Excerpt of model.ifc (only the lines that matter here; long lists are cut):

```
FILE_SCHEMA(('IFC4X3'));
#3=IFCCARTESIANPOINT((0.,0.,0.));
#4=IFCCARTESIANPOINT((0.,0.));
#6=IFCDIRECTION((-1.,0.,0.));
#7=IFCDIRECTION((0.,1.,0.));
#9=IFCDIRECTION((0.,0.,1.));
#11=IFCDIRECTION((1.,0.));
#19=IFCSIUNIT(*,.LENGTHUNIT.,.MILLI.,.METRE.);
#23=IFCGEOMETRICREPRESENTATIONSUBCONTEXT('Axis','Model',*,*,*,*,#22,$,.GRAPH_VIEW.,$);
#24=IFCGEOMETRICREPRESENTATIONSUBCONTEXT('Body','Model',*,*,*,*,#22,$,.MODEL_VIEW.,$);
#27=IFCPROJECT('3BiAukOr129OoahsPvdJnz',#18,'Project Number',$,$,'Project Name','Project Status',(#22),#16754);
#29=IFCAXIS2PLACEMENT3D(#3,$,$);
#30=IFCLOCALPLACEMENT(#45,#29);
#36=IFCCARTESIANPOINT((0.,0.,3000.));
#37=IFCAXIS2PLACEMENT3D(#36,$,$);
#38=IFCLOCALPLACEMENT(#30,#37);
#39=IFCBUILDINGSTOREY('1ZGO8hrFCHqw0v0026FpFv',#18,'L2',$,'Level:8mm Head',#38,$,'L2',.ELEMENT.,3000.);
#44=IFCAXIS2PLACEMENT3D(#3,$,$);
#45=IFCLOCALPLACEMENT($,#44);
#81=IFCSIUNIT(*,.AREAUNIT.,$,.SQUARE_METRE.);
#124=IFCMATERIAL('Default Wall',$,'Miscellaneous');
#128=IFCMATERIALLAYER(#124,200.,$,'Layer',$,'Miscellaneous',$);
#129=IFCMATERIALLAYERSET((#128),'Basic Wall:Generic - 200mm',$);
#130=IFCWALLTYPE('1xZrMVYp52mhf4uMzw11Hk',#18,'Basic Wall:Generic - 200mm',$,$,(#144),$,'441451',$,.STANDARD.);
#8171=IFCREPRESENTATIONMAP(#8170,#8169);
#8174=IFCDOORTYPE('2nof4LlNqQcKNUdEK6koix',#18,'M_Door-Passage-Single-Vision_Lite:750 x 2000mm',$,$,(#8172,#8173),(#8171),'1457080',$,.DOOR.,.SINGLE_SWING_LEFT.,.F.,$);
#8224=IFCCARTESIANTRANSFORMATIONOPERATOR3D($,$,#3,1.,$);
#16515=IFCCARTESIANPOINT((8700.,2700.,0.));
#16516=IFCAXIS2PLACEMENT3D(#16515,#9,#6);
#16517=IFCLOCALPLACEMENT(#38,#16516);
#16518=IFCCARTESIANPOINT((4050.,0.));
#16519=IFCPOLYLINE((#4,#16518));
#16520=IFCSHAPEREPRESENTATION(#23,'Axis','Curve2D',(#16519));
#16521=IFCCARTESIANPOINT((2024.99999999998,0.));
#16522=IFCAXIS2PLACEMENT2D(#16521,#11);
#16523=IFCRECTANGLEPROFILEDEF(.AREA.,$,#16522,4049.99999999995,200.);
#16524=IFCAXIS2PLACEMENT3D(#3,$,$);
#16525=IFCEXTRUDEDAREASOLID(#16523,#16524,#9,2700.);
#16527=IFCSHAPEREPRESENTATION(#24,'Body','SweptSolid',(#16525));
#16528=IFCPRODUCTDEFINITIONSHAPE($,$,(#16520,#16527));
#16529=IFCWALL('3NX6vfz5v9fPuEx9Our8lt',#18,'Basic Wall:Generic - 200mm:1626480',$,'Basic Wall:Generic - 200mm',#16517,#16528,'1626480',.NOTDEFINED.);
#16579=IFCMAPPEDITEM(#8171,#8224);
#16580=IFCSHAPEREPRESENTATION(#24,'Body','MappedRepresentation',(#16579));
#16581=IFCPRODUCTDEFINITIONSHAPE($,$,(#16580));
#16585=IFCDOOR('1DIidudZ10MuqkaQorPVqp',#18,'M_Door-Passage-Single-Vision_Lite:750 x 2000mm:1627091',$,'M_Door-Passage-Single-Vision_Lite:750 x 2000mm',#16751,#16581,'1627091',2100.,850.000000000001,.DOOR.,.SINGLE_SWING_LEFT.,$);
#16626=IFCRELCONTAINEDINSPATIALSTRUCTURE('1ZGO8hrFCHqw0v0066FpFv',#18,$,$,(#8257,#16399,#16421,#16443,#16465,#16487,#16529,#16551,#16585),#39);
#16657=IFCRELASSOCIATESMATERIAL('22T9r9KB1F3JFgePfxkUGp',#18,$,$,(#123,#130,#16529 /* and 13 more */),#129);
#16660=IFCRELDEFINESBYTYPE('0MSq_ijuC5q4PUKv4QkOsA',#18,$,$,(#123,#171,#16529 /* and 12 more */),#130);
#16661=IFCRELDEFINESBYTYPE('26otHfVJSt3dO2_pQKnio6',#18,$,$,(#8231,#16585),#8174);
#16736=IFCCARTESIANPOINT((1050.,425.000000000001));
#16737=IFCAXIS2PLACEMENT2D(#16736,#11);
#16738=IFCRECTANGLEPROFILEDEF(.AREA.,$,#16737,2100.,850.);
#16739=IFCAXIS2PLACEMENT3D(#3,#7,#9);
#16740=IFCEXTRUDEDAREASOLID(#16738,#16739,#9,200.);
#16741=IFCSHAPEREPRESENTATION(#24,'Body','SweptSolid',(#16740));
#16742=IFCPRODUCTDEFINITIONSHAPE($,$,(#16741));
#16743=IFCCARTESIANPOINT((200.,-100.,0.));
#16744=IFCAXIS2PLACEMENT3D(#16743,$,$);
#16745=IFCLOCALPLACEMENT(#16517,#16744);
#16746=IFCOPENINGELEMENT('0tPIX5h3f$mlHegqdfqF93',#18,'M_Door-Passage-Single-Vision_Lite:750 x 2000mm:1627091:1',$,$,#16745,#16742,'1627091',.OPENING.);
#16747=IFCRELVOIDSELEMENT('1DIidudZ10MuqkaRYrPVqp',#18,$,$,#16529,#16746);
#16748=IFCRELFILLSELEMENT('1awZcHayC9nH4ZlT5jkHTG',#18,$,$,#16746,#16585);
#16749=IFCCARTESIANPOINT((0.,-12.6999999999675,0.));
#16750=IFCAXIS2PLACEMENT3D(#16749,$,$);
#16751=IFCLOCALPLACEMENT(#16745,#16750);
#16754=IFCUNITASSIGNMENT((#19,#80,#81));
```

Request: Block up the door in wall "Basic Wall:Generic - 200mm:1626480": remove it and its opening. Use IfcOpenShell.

```python
import ifcopenshell
import ifcopenshell.api.feature
import ifcopenshell.api.root
import ifcopenshell.geom
import ifcopenshell.util.shape

model = ifcopenshell.open("model.ifc")
settings = ifcopenshell.geom.settings()


def volume(element):
    """Net volume in cubic metres, openings subtracted."""
    shape = ifcopenshell.geom.create_shape(settings, element)
    return ifcopenshell.util.shape.get_volume(shape.geometry)


door = model.by_id(16585)
opening = door.FillsVoids[0].RelatingOpeningElement
wall = opening.VoidsElements[0].RelatingBuildingElement
before = volume(wall)

ifcopenshell.api.root.remove_product(model, product=door)
ifcopenshell.api.feature.remove_feature(model, feature=opening)

after = volume(wall)

print(f"wall volume {before:.3f} -> {after:.3f} m3")

model.write("model_updated.ifc")
```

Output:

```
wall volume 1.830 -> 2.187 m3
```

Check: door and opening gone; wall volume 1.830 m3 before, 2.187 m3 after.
